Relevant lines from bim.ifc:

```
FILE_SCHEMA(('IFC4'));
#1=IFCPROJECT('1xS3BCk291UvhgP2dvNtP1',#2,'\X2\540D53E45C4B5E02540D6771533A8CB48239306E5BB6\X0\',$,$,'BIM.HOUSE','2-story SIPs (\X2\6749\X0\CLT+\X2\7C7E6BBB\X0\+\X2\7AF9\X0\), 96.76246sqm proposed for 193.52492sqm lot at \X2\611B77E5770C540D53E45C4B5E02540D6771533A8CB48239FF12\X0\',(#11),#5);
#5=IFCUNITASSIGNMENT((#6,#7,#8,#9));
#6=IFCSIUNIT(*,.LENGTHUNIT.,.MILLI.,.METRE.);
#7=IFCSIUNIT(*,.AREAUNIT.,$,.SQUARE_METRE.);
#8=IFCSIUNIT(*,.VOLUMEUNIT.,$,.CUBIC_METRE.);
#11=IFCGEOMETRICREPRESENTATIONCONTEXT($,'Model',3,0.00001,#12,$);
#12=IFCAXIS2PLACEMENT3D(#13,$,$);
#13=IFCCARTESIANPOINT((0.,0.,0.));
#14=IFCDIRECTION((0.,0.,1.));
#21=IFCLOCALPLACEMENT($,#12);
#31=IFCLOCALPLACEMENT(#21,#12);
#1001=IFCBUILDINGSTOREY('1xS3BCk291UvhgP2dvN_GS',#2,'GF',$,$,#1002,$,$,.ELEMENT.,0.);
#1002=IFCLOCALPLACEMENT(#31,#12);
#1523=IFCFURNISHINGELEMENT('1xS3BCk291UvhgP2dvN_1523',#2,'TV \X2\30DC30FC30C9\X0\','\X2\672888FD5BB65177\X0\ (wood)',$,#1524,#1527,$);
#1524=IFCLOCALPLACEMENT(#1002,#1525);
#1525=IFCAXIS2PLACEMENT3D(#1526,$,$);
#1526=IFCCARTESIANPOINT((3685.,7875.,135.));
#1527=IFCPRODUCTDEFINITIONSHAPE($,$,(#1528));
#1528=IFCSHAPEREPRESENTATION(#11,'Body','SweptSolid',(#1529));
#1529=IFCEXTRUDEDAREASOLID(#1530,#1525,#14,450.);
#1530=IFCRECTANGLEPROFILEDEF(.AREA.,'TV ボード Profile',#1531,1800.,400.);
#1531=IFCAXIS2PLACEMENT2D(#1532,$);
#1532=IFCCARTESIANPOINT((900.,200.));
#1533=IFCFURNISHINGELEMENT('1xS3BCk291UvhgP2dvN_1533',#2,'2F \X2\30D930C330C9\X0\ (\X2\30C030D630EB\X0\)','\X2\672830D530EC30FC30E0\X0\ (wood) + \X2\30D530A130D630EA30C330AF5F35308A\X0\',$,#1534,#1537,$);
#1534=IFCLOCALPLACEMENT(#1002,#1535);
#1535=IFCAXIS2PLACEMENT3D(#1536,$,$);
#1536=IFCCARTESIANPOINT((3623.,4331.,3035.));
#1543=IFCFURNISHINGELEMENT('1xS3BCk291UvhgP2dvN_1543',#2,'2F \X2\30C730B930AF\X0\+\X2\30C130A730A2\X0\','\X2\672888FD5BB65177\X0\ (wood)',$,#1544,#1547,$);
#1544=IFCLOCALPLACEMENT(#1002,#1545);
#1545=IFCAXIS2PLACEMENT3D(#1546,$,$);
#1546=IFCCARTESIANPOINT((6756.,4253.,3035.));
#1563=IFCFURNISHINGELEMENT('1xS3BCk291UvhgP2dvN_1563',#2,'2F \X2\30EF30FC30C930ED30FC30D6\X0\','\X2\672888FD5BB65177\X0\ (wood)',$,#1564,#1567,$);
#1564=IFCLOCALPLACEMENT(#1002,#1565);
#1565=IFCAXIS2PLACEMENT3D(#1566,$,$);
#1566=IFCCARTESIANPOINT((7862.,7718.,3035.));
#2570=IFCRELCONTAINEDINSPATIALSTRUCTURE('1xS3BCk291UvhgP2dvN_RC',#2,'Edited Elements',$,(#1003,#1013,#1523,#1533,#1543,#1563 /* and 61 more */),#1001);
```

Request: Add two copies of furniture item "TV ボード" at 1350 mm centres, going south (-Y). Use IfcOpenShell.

```python
import numpy as np
import ifcopenshell
import ifcopenshell.api.geometry
import ifcopenshell.api.root
import ifcopenshell.util.element
import ifcopenshell.util.placement
import ifcopenshell.util.unit

model = ifcopenshell.open("bim.ifc")
unit_scale = ifcopenshell.util.unit.calculate_unit_scale(model)


def reuse_history(source, copy):
    """copy_class also copies each property set's owner history, people and application; keep the originals."""
    for rel in copy.IsDefinedBy:
        if rel.is_a("IfcRelDefinesByProperties") and (history := rel.RelatingPropertyDefinition.OwnerHistory):
            rel.RelatingPropertyDefinition.OwnerHistory = source.OwnerHistory
            ifcopenshell.util.element.remove_deep2(model, history)


source = model.by_guid("1xS3BCk291UvhgP2dvN_1523")
base = ifcopenshell.util.placement.get_local_placement(source.ObjectPlacement)
step = np.array([0.0, -1.0, 0.0]) * 1.35 / unit_scale

for i in range(1, 3):
    copy = ifcopenshell.api.root.copy_class(model, product=source)
    copy.Representation = ifcopenshell.util.element.copy_deep(
        model, source.Representation, exclude=["IfcGeometricRepresentationContext", "IfcRepresentationMap"]
    )
    reuse_history(source, copy)
    matrix = base.copy()
    matrix[:3, 3] += i * step
    print("added at", matrix[:3, 3].round(3) + 0.0)
    ifcopenshell.api.geometry.edit_object_placement(model, product=copy, matrix=matrix, is_si=False)

model.write("bim_rev.ifc")
```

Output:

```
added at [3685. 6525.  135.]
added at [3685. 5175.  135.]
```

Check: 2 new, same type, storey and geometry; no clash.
